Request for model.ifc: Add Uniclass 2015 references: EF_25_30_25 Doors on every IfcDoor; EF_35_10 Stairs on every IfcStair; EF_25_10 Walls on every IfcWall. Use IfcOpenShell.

First a look at what the model holds.

```python
import ifcopenshell

model = ifcopenshell.open("model.ifc")
print(model.schema)
print("classifications:", [c.Name for c in model.by_type("IfcClassification")])
for ifc_class in ("IfcDoor", "IfcRoof", "IfcStair", "IfcWall", "IfcWindow"):
    print(ifc_class, len(model.by_type(ifc_class)))
```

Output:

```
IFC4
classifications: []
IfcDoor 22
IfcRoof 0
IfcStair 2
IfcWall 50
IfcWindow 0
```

```python
import ifcopenshell
import ifcopenshell.api.classification

model = ifcopenshell.open("model.ifc")

system = ifcopenshell.api.classification.add_classification(model, classification="Uniclass 2015")

codes = {
    "IfcDoor": ("EF_25_30_25", "Doors"),
    "IfcStair": ("EF_35_10", "Stairs"),
    "IfcWall": ("EF_25_10", "Walls"),
}
for ifc_class, (code, name) in codes.items():
    products = model.by_type(ifc_class)
    ifcopenshell.api.classification.add_reference(
        model, products=products, classification=system, identification=code, name=name
    )
    print(code, len(products))

model.write("model-out.ifc")
```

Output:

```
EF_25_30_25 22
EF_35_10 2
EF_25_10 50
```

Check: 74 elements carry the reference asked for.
